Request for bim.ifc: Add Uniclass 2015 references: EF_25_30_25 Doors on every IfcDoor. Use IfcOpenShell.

First a look at what the model holds.

```python
import ifcopenshell

model = ifcopenshell.open("bim.ifc")
print(model.schema)
print("classifications:", [c.Name for c in model.by_type("IfcClassification")])
for ifc_class in ("IfcDoor", "IfcRoof", "IfcStair", "IfcWall", "IfcWindow"):
    print(ifc_class, len(model.by_type(ifc_class)))
```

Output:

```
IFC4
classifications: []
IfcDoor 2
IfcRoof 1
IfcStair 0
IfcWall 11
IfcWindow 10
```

```python
import ifcopenshell
import ifcopenshell.api.classification

model = ifcopenshell.open("bim.ifc")

system = ifcopenshell.api.classification.add_classification(model, classification="Uniclass 2015")

codes = {
    "IfcDoor": ("EF_25_30_25", "Doors"),
}
for ifc_class, (code, name) in codes.items():
    products = model.by_type(ifc_class)
    ifcopenshell.api.classification.add_reference(
        model, products=products, classification=system, identification=code, name=name
    )
    print(code, len(products))

model.write("bim-out.ifc")
```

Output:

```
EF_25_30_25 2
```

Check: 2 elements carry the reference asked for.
